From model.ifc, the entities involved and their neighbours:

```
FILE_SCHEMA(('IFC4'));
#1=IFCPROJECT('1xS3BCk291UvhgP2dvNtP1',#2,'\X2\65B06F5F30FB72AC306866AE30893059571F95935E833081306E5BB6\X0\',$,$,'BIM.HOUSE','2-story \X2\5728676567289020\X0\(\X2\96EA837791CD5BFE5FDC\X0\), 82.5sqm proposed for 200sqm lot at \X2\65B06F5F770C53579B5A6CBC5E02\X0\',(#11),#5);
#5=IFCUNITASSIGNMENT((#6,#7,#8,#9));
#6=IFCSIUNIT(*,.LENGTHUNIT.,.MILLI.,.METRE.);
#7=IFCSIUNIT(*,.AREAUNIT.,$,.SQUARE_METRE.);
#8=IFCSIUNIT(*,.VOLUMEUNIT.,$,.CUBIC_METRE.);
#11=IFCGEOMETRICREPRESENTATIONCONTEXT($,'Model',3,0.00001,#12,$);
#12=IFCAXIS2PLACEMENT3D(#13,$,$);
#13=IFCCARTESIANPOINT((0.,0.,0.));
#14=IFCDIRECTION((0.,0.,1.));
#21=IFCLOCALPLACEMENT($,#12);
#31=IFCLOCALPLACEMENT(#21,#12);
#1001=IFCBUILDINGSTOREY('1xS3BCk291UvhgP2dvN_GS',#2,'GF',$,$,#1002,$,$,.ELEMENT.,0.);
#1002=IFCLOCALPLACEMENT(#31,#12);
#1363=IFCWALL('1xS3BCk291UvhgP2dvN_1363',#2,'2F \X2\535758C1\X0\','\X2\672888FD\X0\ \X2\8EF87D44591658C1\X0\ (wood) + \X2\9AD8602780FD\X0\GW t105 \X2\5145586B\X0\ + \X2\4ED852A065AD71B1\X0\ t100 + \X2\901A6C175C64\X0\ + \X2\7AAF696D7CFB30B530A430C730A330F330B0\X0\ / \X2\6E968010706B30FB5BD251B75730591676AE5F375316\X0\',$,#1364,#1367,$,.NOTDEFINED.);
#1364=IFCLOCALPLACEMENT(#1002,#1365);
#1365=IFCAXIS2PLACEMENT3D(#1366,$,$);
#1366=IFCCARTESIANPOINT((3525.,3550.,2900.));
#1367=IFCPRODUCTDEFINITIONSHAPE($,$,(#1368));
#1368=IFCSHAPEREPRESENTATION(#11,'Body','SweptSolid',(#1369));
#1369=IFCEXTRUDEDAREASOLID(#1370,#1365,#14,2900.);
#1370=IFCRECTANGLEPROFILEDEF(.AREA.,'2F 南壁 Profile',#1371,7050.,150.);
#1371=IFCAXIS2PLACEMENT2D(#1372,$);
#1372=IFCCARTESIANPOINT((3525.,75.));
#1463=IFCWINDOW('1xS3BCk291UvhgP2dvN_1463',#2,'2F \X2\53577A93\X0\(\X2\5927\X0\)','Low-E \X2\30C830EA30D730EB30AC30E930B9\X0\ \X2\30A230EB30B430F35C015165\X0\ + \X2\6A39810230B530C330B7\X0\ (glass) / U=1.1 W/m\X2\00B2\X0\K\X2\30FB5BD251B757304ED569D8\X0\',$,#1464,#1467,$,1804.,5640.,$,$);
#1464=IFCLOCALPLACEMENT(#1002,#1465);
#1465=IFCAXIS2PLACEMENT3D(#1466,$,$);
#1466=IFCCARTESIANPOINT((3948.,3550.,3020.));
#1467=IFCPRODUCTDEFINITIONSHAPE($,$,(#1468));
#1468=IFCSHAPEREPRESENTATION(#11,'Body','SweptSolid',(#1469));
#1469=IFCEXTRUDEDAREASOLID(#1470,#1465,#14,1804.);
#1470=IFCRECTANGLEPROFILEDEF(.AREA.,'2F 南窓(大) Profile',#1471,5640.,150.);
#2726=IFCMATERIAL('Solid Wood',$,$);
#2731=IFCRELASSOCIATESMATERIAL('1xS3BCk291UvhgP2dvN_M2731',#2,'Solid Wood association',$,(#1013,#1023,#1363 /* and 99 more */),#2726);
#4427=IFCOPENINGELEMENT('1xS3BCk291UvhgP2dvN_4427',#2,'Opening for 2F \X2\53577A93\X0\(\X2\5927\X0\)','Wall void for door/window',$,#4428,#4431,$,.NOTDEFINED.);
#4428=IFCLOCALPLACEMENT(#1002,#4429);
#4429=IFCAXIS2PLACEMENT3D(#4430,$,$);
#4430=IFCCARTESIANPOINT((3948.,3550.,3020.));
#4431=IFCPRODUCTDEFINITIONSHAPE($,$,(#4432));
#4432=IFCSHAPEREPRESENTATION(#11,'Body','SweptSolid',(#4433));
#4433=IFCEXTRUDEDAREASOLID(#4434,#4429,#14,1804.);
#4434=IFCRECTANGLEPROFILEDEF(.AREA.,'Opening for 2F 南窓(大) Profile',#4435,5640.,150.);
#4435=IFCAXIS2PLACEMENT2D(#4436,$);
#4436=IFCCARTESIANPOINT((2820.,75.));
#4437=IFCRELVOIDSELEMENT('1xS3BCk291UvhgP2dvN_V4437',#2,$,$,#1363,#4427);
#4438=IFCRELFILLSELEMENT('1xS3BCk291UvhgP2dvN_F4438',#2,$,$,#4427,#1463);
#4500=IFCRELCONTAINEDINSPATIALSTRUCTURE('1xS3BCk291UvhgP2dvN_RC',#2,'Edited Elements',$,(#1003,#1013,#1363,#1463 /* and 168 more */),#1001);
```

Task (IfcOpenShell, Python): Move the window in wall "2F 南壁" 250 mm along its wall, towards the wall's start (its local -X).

```python
import ifcopenshell
import ifcopenshell.api.geometry
import ifcopenshell.util.placement
import ifcopenshell.util.unit

model = ifcopenshell.open("model.ifc")
unit_scale = ifcopenshell.util.unit.calculate_unit_scale(model)

window = model.by_id(1463)
opening = window.FillsVoids[0].RelatingOpeningElement
wall = opening.VoidsElements[0].RelatingBuildingElement

wall_matrix = ifcopenshell.util.placement.get_local_placement(wall.ObjectPlacement)
shift = wall_matrix[:3, 0] * -0.25 / unit_scale
before = ifcopenshell.util.placement.get_local_placement(window.ObjectPlacement)[:3, 3].copy()

# The window is not placed relative to its opening, so move both.
for product in (opening, window):
    matrix = ifcopenshell.util.placement.get_local_placement(product.ObjectPlacement)
    matrix[:3, 3] += shift
    ifcopenshell.api.geometry.edit_object_placement(model, product=product, matrix=matrix, is_si=False)

after = ifcopenshell.util.placement.get_local_placement(window.ObjectPlacement)[:3, 3]
print("window moved by", (after - before).round(3) + 0.0)

model.write("model_edited.ifc")
```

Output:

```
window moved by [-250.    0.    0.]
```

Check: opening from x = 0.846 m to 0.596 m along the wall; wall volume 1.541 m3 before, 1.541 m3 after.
